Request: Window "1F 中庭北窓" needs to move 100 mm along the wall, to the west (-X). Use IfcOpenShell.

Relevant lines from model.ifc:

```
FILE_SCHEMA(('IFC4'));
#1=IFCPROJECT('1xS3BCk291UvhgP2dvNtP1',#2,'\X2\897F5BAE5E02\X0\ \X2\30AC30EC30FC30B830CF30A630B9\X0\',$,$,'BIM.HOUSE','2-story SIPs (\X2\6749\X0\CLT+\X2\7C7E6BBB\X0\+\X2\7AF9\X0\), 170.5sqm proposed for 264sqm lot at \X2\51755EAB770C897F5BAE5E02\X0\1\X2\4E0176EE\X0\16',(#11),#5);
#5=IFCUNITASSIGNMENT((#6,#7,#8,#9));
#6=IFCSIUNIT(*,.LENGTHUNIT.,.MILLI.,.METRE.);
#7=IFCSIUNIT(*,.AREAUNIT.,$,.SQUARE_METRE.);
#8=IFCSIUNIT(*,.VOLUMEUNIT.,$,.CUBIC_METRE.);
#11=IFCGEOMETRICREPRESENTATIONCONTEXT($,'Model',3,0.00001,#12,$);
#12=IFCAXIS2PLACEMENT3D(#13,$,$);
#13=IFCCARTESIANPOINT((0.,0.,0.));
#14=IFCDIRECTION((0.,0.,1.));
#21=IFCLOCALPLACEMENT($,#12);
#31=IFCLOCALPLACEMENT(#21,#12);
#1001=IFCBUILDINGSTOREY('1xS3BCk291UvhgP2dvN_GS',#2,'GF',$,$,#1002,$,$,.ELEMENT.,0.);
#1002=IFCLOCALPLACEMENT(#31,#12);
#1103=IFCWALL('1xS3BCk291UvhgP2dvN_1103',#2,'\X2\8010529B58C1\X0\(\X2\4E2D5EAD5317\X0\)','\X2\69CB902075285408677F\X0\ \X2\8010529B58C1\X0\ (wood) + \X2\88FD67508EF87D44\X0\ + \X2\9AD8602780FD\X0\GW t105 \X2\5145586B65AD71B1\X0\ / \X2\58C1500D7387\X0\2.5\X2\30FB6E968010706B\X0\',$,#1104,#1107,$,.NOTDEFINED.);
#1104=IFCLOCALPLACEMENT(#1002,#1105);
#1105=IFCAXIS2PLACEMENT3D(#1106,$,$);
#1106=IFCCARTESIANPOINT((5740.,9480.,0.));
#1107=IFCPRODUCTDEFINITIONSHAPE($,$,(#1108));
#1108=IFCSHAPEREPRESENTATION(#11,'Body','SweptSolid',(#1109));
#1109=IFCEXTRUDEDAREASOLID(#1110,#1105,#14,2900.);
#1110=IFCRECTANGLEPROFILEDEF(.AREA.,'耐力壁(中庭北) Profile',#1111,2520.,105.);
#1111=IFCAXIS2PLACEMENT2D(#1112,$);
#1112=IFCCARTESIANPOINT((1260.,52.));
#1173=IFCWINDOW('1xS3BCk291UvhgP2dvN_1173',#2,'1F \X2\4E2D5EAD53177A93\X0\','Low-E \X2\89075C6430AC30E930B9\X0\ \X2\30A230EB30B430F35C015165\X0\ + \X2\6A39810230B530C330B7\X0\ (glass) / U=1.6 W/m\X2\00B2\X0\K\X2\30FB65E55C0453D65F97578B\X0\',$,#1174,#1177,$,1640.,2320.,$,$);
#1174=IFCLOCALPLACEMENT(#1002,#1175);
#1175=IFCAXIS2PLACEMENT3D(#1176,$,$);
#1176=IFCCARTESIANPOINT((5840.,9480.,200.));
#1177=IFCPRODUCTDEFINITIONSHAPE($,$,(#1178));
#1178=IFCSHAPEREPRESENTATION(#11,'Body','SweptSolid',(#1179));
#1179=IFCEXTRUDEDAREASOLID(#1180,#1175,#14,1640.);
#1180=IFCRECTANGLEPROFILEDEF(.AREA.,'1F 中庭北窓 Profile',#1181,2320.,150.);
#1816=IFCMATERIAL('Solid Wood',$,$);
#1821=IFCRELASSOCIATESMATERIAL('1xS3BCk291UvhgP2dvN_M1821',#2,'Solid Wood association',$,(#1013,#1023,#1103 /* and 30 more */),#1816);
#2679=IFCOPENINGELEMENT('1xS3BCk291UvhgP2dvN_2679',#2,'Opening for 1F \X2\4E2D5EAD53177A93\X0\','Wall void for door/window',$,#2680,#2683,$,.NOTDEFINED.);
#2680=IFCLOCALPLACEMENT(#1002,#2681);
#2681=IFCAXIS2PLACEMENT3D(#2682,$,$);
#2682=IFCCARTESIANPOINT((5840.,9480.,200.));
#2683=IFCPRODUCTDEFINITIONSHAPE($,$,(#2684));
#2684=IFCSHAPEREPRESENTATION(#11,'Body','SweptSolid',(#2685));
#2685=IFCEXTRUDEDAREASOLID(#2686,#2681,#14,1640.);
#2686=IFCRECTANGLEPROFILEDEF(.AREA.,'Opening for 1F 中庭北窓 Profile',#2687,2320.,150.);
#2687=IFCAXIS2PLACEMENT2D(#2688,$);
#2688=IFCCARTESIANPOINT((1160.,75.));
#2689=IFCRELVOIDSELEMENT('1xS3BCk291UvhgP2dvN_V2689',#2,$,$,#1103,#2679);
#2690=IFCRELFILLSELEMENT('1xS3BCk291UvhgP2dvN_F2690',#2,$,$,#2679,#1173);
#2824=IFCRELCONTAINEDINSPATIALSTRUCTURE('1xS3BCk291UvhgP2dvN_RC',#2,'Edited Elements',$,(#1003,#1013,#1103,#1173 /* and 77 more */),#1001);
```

```python
import ifcopenshell
import ifcopenshell.api.geometry
import ifcopenshell.util.placement

model = ifcopenshell.open("model.ifc")

window = model.by_guid("1xS3BCk291UvhgP2dvN_1173")
opening = window.FillsVoids[0].RelatingOpeningElement
wall = opening.VoidsElements[0].RelatingBuildingElement

wall_matrix = ifcopenshell.util.placement.get_local_placement(wall.ObjectPlacement)
shift = wall_matrix[:3, 0] * -100.0
before = ifcopenshell.util.placement.get_local_placement(window.ObjectPlacement)[:3, 3].copy()

# The window is not placed relative to its opening, so move both.
for product in (opening, window):
    matrix = ifcopenshell.util.placement.get_local_placement(product.ObjectPlacement)
    matrix[:3, 3] += shift
    ifcopenshell.api.geometry.edit_object_placement(model, product=product, matrix=matrix, is_si=False)

after = ifcopenshell.util.placement.get_local_placement(window.ObjectPlacement)[:3, 3]
print("window moved by", (after - before).round(3) + 0.0)

model.write("model_rev.ifc")
```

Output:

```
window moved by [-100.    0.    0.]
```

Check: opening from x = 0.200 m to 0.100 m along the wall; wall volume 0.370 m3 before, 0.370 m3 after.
